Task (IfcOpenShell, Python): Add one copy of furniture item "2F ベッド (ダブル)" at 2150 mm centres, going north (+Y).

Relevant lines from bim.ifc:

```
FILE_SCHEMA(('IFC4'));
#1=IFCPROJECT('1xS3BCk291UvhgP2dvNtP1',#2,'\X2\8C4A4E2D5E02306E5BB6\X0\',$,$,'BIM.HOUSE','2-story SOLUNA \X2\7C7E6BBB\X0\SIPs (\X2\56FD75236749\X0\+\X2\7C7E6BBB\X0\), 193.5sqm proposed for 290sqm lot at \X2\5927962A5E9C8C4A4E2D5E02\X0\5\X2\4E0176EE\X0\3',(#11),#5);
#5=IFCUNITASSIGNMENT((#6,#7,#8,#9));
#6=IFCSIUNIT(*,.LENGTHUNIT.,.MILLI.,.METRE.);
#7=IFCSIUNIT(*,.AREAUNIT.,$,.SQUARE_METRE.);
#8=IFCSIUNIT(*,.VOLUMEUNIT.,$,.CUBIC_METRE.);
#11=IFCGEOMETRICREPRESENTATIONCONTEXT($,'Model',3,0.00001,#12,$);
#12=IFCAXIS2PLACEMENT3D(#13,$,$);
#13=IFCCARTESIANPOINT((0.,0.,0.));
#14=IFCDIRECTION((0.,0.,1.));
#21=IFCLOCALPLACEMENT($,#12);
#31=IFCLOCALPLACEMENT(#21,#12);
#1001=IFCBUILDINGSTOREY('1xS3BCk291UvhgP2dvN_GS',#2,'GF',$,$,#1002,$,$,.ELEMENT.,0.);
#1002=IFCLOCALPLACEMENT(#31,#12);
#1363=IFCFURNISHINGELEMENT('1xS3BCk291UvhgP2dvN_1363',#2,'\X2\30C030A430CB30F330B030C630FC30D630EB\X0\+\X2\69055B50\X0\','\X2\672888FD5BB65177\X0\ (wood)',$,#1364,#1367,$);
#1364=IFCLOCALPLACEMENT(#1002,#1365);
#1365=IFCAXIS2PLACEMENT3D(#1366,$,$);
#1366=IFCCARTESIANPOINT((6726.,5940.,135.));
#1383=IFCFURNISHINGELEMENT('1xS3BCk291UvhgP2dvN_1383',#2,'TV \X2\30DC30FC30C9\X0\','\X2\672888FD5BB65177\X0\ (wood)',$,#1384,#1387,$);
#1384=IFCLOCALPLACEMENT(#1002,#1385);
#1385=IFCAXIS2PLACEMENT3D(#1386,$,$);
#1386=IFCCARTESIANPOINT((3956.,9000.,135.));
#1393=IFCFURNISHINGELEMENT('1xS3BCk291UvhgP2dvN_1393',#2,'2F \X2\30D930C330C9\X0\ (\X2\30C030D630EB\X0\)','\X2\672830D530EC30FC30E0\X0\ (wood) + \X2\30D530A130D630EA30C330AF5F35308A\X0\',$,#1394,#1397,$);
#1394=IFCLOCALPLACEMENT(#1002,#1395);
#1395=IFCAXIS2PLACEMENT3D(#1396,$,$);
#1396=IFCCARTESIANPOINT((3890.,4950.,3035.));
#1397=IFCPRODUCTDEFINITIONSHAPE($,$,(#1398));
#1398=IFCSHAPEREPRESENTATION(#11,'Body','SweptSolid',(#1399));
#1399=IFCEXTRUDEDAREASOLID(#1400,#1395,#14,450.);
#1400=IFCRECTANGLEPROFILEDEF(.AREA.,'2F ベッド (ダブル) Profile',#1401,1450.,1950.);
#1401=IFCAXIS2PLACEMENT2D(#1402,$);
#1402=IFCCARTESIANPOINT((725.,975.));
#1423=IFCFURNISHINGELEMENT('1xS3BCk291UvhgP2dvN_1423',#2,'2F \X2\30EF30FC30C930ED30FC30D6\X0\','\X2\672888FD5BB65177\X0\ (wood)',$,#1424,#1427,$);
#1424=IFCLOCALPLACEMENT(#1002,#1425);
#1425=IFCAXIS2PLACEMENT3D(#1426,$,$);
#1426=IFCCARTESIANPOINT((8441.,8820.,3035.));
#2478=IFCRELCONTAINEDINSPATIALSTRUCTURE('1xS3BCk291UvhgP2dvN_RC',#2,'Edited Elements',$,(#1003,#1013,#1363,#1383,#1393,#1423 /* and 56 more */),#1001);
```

```python
import numpy as np
import ifcopenshell
import ifcopenshell.api.geometry
import ifcopenshell.api.root
import ifcopenshell.util.element
import ifcopenshell.util.placement
import ifcopenshell.util.unit

model = ifcopenshell.open("bim.ifc")
unit_scale = ifcopenshell.util.unit.calculate_unit_scale(model)


def reuse_history(source, copy):
    """copy_class also copies each property set's owner history, people and application; keep the originals."""
    for rel in copy.IsDefinedBy:
        if rel.is_a("IfcRelDefinesByProperties") and (history := rel.RelatingPropertyDefinition.OwnerHistory):
            rel.RelatingPropertyDefinition.OwnerHistory = source.OwnerHistory
            ifcopenshell.util.element.remove_deep2(model, history)


source = model.by_id(1393)
base = ifcopenshell.util.placement.get_local_placement(source.ObjectPlacement)
step = np.array([0.0, 1.0, 0.0]) * 2.15 / unit_scale

for i in range(1, 2):
    copy = ifcopenshell.api.root.copy_class(model, product=source)
    copy.Representation = ifcopenshell.util.element.copy_deep(
        model, source.Representation, exclude=["IfcGeometricRepresentationContext", "IfcRepresentationMap"]
    )
    reuse_history(source, copy)
    matrix = base.copy()
    matrix[:3, 3] += i * step
    print("added at", matrix[:3, 3].round(3) + 0.0)
    ifcopenshell.api.geometry.edit_object_placement(model, product=copy, matrix=matrix, is_si=False)

model.write("bim_v2.ifc")
```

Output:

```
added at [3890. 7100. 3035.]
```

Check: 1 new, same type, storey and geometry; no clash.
